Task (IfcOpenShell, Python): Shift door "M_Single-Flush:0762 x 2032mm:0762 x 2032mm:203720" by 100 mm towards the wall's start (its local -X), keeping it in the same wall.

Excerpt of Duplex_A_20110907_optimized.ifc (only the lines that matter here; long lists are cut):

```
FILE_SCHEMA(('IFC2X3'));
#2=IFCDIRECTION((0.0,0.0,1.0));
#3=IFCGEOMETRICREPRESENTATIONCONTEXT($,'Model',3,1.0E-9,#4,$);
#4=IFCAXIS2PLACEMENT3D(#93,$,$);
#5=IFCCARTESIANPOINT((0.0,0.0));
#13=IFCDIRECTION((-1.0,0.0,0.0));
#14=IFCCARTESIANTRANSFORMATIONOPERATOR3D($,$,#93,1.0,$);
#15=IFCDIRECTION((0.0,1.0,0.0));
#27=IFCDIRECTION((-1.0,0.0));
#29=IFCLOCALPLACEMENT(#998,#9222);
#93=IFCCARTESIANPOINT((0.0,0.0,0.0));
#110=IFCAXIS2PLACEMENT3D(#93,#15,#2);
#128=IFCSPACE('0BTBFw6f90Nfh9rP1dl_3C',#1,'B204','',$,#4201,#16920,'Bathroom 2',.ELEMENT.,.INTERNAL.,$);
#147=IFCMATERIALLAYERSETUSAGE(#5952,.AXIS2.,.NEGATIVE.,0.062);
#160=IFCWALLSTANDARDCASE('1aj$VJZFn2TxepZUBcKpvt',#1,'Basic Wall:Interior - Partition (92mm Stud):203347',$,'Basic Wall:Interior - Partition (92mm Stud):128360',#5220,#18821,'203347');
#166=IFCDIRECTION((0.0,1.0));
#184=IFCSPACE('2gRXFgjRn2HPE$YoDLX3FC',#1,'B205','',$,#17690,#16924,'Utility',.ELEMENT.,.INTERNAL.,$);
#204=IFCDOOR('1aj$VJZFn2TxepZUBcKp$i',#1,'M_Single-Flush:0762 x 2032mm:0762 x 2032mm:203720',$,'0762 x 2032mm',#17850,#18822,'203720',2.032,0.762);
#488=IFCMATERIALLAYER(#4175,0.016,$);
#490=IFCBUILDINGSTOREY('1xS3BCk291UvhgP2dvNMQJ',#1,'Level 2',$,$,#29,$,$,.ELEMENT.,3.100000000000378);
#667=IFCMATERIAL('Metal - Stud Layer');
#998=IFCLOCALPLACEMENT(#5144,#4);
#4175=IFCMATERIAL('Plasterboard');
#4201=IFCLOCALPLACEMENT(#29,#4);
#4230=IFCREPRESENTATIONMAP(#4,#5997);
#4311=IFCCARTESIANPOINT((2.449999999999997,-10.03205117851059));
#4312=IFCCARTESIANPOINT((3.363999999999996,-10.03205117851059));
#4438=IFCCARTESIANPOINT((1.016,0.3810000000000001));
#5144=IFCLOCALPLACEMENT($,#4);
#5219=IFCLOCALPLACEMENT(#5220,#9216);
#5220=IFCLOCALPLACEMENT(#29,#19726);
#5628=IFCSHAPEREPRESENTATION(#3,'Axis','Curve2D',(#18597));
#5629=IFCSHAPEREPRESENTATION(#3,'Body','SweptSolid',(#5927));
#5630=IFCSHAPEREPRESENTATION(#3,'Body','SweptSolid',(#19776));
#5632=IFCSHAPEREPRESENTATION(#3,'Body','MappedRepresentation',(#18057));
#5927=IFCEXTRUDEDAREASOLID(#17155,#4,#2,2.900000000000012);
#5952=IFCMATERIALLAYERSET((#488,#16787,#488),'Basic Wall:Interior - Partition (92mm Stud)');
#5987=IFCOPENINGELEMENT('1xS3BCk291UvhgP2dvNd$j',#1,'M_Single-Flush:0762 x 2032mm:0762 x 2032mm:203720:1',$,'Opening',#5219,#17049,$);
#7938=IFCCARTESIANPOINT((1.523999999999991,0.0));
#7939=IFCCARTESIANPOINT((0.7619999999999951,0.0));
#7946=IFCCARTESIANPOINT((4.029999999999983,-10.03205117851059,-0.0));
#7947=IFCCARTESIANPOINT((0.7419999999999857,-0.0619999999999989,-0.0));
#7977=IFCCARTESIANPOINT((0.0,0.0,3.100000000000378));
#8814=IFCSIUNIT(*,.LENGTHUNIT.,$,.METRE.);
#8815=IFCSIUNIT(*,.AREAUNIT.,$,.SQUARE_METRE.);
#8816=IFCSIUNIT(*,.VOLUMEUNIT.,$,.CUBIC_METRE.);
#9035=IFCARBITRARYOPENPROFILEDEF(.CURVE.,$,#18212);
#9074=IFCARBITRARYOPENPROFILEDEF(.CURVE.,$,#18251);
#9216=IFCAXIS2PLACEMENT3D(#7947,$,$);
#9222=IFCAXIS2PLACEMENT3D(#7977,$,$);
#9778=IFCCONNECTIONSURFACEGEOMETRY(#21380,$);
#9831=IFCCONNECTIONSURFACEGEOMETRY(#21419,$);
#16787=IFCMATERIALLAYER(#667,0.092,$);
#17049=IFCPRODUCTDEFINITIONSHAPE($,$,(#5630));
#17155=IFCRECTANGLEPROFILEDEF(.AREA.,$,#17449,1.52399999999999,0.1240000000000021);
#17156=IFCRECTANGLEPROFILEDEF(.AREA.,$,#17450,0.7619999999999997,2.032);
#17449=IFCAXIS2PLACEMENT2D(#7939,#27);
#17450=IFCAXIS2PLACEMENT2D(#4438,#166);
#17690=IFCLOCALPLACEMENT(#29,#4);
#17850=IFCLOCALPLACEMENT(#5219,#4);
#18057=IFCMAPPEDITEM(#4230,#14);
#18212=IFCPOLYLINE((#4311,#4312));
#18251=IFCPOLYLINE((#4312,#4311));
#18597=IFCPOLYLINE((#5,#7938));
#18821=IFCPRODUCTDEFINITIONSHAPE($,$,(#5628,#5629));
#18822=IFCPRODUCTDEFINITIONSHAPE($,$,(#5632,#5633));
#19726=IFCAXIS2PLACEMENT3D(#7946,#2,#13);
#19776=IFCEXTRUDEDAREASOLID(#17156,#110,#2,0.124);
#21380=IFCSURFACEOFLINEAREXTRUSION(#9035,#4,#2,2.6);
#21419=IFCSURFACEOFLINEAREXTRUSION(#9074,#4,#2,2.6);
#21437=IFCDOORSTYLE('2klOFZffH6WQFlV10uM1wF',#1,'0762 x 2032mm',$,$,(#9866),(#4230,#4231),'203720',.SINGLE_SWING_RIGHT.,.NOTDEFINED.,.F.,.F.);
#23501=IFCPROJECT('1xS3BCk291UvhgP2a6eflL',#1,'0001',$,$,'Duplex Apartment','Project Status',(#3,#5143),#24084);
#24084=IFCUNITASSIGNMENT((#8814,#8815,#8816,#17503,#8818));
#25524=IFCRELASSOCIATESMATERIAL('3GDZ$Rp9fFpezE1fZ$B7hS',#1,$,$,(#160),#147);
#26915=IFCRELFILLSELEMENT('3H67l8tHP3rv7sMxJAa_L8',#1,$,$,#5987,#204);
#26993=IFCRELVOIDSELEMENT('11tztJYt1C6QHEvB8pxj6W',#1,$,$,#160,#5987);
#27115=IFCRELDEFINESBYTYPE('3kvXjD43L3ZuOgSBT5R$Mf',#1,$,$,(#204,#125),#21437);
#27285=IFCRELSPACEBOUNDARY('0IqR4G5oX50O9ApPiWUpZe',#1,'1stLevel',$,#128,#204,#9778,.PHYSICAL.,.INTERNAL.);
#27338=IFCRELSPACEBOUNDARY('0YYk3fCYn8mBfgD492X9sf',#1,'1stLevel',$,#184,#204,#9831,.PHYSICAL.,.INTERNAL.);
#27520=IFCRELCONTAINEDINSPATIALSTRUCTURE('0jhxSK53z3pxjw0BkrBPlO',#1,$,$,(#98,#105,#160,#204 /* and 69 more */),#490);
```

```python
import numpy as np
import ifcopenshell
import ifcopenshell.api.geometry
import ifcopenshell.util.placement
import ifcopenshell.util.unit

model = ifcopenshell.open("Duplex_A_20110907_optimized.ifc")
unit_scale = ifcopenshell.util.unit.calculate_unit_scale(model)

door = model.by_guid("1aj$VJZFn2TxepZUBcKp$i")
opening = door.FillsVoids[0].RelatingOpeningElement
wall = opening.VoidsElements[0].RelatingBuildingElement

wall_matrix = ifcopenshell.util.placement.get_local_placement(wall.ObjectPlacement)
shift = wall_matrix[:3, 0] * -0.1 / unit_scale
before = ifcopenshell.util.placement.get_local_placement(door.ObjectPlacement)[:3, 3].copy()

# The door is placed relative to its opening, so it follows when the opening moves.
matrix = ifcopenshell.util.placement.get_local_placement(opening.ObjectPlacement)
matrix[:3, 3] += shift
ifcopenshell.api.geometry.edit_object_placement(
    model, product=opening, matrix=matrix, is_si=False, should_transform_children=True
)

# Space boundary surfaces are stored in each space's coordinates; move them too.
for rel in door.ProvidesBoundaries:
    if not rel.ConnectionGeometry:
        continue
    surface = rel.ConnectionGeometry.SurfaceOnRelatingElement
    space_matrix = ifcopenshell.util.placement.get_local_placement(rel.RelatingSpace.ObjectPlacement)
    point = np.array(surface.Position.Location.Coordinates) + space_matrix[:3, :3].T @ shift
    surface.Position = model.createIfcAxis2Placement3D(
        model.createIfcCartesianPoint(point.tolist()), surface.Position.Axis, surface.Position.RefDirection
    )

after = ifcopenshell.util.placement.get_local_placement(door.ObjectPlacement)[:3, 3]
print("door moved by", (after - before).round(3) + 0.0)

model.write("Duplex_A_20110907_optimized-out.ifc")
```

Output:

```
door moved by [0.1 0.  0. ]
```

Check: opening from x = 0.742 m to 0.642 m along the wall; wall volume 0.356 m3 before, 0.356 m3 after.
